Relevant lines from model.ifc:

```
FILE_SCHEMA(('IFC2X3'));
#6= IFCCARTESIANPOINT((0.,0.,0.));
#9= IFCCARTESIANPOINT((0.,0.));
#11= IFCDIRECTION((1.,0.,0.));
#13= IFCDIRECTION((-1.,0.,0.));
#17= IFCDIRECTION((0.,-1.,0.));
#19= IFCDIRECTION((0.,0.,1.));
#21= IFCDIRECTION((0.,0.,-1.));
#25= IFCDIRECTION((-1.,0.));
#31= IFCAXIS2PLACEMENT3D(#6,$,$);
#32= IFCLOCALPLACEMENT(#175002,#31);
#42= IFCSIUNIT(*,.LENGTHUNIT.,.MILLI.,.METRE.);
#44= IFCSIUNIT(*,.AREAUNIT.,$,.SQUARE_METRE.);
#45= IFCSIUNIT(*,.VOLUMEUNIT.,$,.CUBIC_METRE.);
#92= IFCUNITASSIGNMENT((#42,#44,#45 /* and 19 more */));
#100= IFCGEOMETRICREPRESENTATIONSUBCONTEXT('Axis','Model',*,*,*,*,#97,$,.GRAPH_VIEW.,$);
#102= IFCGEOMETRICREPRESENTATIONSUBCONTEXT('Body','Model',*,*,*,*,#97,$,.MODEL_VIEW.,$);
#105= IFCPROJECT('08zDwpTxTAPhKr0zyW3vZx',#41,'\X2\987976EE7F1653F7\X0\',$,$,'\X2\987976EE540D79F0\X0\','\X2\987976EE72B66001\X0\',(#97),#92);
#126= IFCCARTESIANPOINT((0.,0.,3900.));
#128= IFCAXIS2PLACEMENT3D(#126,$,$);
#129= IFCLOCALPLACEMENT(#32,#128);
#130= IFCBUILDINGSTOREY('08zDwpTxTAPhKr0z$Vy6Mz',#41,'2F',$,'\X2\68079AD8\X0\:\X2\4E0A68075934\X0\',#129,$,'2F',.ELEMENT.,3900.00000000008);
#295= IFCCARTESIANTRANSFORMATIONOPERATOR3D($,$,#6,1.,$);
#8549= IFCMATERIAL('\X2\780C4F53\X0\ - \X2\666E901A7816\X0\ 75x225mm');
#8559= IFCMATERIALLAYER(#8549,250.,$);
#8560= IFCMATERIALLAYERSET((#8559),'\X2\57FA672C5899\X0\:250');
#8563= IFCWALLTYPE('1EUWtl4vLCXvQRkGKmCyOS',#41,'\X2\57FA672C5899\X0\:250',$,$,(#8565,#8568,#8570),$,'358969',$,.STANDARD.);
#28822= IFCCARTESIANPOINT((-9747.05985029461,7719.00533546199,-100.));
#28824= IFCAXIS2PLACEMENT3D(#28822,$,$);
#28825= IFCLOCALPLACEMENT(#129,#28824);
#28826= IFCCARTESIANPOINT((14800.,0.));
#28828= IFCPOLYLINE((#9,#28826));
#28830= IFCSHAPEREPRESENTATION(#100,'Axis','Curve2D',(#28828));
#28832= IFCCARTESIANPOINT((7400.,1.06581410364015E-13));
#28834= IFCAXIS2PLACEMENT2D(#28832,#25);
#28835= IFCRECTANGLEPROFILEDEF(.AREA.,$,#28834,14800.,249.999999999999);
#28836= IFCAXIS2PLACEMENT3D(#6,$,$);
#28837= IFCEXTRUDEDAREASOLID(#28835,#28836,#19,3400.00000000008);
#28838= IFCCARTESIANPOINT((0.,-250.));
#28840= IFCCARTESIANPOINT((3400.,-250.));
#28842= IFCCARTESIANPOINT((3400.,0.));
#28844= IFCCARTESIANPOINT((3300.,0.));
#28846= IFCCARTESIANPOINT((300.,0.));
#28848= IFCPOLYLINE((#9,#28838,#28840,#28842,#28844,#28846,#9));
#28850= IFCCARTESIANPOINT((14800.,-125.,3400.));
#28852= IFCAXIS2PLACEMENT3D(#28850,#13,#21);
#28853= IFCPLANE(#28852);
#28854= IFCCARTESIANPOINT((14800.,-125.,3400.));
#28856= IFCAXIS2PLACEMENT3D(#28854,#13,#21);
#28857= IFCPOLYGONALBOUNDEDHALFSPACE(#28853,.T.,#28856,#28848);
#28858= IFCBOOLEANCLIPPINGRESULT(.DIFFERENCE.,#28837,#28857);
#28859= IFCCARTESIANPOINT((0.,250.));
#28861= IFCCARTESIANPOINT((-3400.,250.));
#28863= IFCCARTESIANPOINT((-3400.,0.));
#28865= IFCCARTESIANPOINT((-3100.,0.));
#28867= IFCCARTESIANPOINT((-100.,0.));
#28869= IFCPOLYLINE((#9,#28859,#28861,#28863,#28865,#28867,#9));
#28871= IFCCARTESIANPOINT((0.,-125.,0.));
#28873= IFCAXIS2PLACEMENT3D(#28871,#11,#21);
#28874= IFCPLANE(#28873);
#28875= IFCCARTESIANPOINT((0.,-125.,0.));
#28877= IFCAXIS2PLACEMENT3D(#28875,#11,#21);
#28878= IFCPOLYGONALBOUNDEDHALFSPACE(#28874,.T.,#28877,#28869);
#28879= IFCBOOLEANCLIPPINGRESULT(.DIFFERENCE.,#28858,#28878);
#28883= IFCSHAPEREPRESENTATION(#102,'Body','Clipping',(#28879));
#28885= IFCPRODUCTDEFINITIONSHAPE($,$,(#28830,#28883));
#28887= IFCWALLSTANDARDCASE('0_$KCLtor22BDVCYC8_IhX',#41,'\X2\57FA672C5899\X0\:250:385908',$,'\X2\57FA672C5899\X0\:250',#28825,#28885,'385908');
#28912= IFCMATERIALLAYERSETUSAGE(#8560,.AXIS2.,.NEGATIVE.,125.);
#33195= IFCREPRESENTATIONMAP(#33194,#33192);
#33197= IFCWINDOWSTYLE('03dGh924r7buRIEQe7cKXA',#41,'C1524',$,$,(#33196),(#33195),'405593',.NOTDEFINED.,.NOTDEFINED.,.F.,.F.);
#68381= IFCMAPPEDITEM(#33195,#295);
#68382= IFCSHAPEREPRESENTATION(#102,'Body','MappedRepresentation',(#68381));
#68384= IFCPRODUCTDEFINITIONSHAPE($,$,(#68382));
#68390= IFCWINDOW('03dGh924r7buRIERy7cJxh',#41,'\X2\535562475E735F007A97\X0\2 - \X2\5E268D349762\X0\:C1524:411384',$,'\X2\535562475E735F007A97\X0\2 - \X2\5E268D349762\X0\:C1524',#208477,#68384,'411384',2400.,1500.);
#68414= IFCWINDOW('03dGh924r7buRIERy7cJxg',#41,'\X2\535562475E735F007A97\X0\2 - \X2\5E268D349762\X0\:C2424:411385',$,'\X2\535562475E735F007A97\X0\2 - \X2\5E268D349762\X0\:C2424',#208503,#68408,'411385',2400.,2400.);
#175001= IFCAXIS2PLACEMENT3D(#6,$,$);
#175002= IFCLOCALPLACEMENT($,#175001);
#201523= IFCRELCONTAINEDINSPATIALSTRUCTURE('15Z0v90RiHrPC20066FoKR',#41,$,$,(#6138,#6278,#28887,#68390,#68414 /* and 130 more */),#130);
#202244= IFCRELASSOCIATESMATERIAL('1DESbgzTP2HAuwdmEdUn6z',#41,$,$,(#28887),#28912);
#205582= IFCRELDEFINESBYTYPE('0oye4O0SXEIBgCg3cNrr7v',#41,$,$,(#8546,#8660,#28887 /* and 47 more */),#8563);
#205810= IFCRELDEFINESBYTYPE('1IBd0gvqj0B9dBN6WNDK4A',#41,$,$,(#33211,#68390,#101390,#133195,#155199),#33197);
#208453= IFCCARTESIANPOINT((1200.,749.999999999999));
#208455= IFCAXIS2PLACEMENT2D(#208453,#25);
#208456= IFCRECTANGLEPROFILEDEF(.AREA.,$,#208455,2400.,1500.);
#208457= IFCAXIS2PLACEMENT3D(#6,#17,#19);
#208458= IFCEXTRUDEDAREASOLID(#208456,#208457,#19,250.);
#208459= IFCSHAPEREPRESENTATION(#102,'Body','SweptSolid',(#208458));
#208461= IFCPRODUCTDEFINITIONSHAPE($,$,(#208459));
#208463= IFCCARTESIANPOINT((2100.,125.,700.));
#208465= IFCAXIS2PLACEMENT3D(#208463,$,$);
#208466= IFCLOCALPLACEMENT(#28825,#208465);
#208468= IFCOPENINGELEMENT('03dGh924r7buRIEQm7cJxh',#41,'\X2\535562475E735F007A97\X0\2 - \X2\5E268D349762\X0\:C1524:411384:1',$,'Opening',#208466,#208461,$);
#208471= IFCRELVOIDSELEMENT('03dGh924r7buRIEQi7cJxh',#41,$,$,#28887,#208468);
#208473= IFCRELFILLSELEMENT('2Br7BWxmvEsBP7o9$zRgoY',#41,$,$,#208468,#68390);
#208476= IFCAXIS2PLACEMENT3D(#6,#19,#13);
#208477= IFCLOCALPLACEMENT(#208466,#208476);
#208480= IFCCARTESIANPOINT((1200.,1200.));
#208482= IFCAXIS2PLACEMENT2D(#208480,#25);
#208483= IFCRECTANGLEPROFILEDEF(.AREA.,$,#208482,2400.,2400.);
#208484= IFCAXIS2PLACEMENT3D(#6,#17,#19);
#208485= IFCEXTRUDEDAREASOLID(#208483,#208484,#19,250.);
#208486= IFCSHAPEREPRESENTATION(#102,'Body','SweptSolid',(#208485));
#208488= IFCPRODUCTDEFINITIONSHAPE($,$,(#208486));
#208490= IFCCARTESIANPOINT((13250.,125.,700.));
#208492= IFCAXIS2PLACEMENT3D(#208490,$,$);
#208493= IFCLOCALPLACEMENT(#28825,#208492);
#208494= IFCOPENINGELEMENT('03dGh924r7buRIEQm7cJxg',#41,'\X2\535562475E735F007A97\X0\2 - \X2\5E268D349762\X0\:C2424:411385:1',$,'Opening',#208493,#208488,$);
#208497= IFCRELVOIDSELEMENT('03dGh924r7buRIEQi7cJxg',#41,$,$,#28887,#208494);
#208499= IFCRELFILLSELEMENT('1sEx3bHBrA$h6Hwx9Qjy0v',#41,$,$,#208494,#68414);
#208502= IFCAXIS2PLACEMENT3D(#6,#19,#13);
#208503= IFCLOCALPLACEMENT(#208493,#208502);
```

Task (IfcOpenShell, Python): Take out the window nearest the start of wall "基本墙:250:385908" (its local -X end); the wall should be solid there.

```python
import ifcopenshell
import ifcopenshell.api.feature
import ifcopenshell.api.root
import ifcopenshell.geom
import ifcopenshell.util.shape

model = ifcopenshell.open("model.ifc")
settings = ifcopenshell.geom.settings()


def volume(element):
    """Net volume in cubic metres, openings subtracted."""
    shape = ifcopenshell.geom.create_shape(settings, element)
    return ifcopenshell.util.shape.get_volume(shape.geometry)


window = model.by_guid("03dGh924r7buRIERy7cJxh")
opening = window.FillsVoids[0].RelatingOpeningElement
wall = opening.VoidsElements[0].RelatingBuildingElement
before = volume(wall)

ifcopenshell.api.root.remove_product(model, product=window)
ifcopenshell.api.feature.remove_feature(model, feature=opening)

after = volume(wall)

print(f"wall volume {before:.3f} -> {after:.3f} m3")

model.write("model_v2.ifc")
```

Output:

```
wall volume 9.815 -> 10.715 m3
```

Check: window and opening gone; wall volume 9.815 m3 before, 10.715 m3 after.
